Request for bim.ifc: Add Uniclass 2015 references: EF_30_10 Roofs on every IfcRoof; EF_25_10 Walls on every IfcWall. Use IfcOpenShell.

First a look at what the model holds.

```python
import ifcopenshell

model = ifcopenshell.open("bim.ifc")
print(model.schema)
print("classifications:", [c.Name for c in model.by_type("IfcClassification")])
for ifc_class in ("IfcDoor", "IfcRoof", "IfcStair", "IfcWall", "IfcWindow"):
    print(ifc_class, len(model.by_type(ifc_class)))
```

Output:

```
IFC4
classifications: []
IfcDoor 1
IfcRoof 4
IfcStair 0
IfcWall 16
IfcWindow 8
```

```python
import ifcopenshell
import ifcopenshell.api.classification

model = ifcopenshell.open("bim.ifc")

system = ifcopenshell.api.classification.add_classification(model, classification="Uniclass 2015")

codes = {
    "IfcRoof": ("EF_30_10", "Roofs"),
    "IfcWall": ("EF_25_10", "Walls"),
}
for ifc_class, (code, name) in codes.items():
    products = model.by_type(ifc_class)
    ifcopenshell.api.classification.add_reference(
        model, products=products, classification=system, identification=code, name=name
    )
    print(code, len(products))

model.write("bim_rev.ifc")
```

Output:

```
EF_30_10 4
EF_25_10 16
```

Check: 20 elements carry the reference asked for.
